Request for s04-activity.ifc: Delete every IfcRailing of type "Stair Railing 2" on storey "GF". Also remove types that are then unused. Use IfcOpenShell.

First a look at what the model holds.

```python
import ifcopenshell
import ifcopenshell.util.element

model = ifcopenshell.open("s04-activity.ifc")
print(model.schema)
storey = next(s for s in model.by_type("IfcBuildingStorey") if s.Name == "GF")
railings = [e for e in ifcopenshell.util.element.get_decomposition(storey) if e.is_a("IfcRailing")]
seen = {}
for e in railings:
    element_type = ifcopenshell.util.element.get_type(e)
    name = element_type.Name if element_type not in (None, e) else None
    seen[name] = seen.get(name, 0) + 1
for name, count in sorted(seen.items(), key=str):
    print(count, "x", name)
```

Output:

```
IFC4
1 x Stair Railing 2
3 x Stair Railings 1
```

```python
import ifcopenshell
import ifcopenshell.api.root
import ifcopenshell.util.element

model = ifcopenshell.open("s04-activity.ifc")

storey = next(s for s in model.by_type("IfcBuildingStorey") if s.Name == "GF")
railings = [e for e in ifcopenshell.util.element.get_decomposition(storey) if e.is_a("IfcRailing")]
targets = [e for e in railings if (t := ifcopenshell.util.element.get_type(e)) not in (None, e) and t.Name == "Stair Railing 2"]
types = {ifcopenshell.util.element.get_type(e) for e in targets} - {None, *targets}

for e in targets:
    ifcopenshell.api.root.remove_product(model, product=e)
print(len(targets), "removed")

unused = [t for t in types if not ifcopenshell.util.element.get_types(t)]
for t in unused:
    ifcopenshell.api.root.remove_product(model, product=t)
print(len(unused), "unused types removed")

model.write("s04-activity_v2.ifc")
```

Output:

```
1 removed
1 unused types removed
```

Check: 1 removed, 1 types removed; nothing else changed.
